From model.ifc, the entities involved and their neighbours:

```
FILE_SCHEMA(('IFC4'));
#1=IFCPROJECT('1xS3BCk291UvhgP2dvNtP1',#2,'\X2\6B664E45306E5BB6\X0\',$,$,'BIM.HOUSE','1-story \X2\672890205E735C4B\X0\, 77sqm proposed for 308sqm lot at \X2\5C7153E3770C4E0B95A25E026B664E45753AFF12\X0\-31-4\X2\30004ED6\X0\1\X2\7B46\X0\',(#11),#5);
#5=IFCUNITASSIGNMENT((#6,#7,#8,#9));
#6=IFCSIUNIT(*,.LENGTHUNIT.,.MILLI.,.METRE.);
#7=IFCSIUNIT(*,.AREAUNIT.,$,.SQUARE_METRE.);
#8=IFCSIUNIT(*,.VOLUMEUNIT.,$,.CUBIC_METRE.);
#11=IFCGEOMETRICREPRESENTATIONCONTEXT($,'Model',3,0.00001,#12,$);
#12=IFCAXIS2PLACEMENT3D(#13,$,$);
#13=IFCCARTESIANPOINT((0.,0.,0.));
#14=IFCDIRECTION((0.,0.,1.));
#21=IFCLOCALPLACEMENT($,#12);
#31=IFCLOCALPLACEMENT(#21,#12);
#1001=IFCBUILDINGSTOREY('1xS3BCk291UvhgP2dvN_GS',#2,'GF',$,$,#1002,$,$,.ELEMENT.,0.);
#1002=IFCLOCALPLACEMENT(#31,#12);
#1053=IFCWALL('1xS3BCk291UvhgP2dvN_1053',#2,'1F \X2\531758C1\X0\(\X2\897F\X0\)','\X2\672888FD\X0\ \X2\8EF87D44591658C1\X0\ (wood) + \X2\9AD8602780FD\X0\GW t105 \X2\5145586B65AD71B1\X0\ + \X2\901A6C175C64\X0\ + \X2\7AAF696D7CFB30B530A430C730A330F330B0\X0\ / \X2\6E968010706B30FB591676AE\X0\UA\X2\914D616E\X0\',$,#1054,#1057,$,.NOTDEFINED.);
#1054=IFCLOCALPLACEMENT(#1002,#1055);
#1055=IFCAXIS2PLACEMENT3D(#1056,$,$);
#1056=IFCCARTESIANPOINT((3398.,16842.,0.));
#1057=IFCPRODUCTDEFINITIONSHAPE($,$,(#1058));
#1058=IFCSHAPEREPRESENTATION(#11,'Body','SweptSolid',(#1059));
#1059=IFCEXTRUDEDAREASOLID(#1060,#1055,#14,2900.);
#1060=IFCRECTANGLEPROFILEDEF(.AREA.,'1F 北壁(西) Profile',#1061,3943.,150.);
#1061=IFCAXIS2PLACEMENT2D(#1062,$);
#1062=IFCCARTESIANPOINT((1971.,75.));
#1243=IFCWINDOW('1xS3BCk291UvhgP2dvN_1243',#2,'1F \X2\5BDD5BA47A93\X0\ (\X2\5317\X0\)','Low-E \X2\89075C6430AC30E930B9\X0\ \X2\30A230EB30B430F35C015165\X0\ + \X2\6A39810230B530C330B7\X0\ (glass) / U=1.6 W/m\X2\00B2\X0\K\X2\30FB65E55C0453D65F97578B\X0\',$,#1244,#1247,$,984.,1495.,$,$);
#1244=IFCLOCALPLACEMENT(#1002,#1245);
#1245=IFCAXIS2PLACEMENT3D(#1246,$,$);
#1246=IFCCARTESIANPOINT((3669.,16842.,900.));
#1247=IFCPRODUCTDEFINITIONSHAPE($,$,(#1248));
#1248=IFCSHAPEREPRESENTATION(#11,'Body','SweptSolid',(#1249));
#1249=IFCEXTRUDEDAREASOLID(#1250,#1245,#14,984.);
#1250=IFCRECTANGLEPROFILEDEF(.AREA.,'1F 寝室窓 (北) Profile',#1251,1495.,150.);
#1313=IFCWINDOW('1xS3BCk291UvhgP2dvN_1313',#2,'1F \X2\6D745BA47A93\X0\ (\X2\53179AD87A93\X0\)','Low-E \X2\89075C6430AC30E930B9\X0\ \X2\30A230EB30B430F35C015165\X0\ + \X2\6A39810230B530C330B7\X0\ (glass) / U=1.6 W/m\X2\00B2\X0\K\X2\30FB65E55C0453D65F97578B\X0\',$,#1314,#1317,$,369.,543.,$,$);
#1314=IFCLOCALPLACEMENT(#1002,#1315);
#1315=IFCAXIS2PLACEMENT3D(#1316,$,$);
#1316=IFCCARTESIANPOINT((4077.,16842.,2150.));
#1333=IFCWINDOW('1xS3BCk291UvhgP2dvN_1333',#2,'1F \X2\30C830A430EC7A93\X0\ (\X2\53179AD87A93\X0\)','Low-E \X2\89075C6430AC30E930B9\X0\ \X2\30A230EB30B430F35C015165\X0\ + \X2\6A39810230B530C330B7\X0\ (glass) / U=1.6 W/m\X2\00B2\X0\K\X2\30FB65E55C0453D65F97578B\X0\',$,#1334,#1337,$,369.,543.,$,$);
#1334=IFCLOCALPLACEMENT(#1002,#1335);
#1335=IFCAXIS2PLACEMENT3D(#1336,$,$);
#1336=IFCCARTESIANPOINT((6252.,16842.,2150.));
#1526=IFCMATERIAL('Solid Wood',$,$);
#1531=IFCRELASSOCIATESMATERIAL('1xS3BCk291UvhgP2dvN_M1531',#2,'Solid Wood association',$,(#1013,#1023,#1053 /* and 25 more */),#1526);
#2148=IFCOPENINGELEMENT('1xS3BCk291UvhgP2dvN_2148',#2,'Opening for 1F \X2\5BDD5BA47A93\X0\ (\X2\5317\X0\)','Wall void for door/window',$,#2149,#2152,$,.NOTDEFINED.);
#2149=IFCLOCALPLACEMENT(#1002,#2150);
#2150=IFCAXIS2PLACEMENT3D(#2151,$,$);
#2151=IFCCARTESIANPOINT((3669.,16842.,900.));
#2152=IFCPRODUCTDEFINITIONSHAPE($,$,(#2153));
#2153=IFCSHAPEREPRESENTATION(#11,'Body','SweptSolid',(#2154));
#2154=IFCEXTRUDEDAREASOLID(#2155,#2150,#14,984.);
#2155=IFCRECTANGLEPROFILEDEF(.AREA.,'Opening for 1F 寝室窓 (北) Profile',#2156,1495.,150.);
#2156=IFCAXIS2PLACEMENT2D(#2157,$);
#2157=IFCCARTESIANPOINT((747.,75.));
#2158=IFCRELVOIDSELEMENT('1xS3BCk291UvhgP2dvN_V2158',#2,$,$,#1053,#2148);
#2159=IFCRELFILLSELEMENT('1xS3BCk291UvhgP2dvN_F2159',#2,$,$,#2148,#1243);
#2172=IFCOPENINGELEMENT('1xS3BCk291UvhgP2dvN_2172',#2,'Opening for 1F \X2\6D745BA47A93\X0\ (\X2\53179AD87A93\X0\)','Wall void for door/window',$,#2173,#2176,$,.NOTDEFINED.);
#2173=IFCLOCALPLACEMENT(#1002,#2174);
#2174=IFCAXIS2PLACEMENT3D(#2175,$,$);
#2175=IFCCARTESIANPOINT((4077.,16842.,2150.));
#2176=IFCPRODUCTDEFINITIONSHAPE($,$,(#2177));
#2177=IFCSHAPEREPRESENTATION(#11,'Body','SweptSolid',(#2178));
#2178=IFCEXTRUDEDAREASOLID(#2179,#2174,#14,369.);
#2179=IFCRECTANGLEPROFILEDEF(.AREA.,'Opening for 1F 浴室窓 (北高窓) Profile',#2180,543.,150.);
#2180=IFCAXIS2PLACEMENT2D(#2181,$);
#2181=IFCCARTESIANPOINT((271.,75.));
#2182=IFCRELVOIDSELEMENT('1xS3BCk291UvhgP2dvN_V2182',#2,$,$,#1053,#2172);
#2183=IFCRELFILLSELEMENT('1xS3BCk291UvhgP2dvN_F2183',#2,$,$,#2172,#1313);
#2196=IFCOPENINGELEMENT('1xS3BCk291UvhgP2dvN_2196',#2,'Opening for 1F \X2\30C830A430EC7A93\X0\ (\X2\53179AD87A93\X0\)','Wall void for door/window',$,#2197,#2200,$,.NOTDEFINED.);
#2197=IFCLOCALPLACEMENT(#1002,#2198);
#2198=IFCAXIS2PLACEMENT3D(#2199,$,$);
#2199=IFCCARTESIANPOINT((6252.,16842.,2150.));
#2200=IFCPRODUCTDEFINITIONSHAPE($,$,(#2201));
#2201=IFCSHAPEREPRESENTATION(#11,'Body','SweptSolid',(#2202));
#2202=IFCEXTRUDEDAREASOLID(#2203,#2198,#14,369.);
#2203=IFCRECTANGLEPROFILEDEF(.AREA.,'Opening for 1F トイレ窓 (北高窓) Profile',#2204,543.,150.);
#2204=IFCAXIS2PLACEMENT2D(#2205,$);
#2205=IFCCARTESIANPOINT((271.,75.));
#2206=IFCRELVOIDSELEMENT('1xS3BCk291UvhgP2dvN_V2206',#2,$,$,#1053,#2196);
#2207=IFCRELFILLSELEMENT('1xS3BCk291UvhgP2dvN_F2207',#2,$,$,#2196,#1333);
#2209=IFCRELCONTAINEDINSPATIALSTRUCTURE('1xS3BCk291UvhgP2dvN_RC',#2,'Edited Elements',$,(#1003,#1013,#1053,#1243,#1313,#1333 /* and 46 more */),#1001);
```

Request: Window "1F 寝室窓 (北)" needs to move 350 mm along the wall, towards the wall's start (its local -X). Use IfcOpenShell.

```python
import ifcopenshell
import ifcopenshell.api.geometry
import ifcopenshell.util.placement

model = ifcopenshell.open("model.ifc")

window = model.by_id(1243)
opening = window.FillsVoids[0].RelatingOpeningElement
wall = opening.VoidsElements[0].RelatingBuildingElement

wall_matrix = ifcopenshell.util.placement.get_local_placement(wall.ObjectPlacement)
shift = wall_matrix[:3, 0] * -350.0
before = ifcopenshell.util.placement.get_local_placement(window.ObjectPlacement)[:3, 3].copy()

# The window is not placed relative to its opening, so move both.
for product in (opening, window):
    matrix = ifcopenshell.util.placement.get_local_placement(product.ObjectPlacement)
    matrix[:3, 3] += shift
    ifcopenshell.api.geometry.edit_object_placement(model, product=product, matrix=matrix, is_si=False)

after = ifcopenshell.util.placement.get_local_placement(window.ObjectPlacement)[:3, 3]
print("window moved by", (after - before).round(3) + 0.0)

model.write("model_rev.ifc")
```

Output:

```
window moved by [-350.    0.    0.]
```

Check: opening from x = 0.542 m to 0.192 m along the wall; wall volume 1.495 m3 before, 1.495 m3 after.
